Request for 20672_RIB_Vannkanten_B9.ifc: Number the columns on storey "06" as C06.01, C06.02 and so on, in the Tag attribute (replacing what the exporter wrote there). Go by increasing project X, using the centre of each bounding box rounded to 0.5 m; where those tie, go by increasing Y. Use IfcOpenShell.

First a look at what the model holds.

```python
import ifcopenshell
import ifcopenshell.util.element
import ifcopenshell.util.placement

model = ifcopenshell.open("20672_RIB_Vannkanten_B9.ifc")
print(model.schema)
storey = next(s for s in model.by_type("IfcBuildingStorey") if s.Name == "06")
columns = [e for e in ifcopenshell.util.element.get_decomposition(storey) if e.is_a("IfcColumn")]
for e in sorted(columns, key=lambda e: e.id()):
    origin = ifcopenshell.util.placement.get_local_placement(e.ObjectPlacement)[:3, 3]
    print(e.id(), e.Tag, e.Name, origin.round(2) + 0.0, sep=" | ")
```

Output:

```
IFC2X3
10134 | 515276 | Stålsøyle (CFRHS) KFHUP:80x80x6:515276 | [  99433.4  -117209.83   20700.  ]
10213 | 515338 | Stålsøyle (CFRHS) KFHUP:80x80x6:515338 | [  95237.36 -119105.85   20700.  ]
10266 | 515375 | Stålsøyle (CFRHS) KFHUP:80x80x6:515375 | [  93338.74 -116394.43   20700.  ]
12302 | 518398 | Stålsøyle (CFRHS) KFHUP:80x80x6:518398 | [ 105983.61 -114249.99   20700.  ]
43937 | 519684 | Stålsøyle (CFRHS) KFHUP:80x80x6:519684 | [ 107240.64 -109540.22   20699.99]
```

```python
import ifcopenshell
import ifcopenshell.geom
import ifcopenshell.util.element
import ifcopenshell.util.shape

model = ifcopenshell.open("20672_RIB_Vannkanten_B9.ifc")
settings = ifcopenshell.geom.settings()
settings.set("use-world-coords", True)


def centre(element):
    shape = ifcopenshell.geom.create_shape(settings, element)
    return ifcopenshell.util.shape.get_bbox_centroid(shape.geometry)


storey = next(s for s in model.by_type("IfcBuildingStorey") if s.Name == "06")
columns = [e for e in ifcopenshell.util.element.get_decomposition(storey) if e.is_a("IfcColumn")]

# Insertion points can sit at a corner or the storey origin, so sort by the geometry (in metres).
centres = {e: centre(e) for e in columns}
columns.sort(key=lambda e: (round(centres[e][0] / 0.5), centres[e][1]))

for i, e in enumerate(columns, start=1):
    number = f"C06.{i:02d}"
    e.Tag = number
    print(e.id(), number)

model.write("20672_RIB_Vannkanten_B9_v2.ifc")
```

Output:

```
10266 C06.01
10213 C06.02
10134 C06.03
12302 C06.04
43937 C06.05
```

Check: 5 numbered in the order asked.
